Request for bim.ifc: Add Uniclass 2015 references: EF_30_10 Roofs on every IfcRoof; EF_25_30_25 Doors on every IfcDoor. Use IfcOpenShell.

First a look at what the model holds.

```python
import ifcopenshell

model = ifcopenshell.open("bim.ifc")
print(model.schema)
print("classifications:", [c.Name for c in model.by_type("IfcClassification")])
for ifc_class in ("IfcDoor", "IfcRoof", "IfcStair", "IfcWall", "IfcWindow"):
    print(ifc_class, len(model.by_type(ifc_class)))
```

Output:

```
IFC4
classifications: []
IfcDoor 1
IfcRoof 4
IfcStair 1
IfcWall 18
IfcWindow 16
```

```python
import ifcopenshell
import ifcopenshell.api.classification

model = ifcopenshell.open("bim.ifc")

system = ifcopenshell.api.classification.add_classification(model, classification="Uniclass 2015")

codes = {
    "IfcRoof": ("EF_30_10", "Roofs"),
    "IfcDoor": ("EF_25_30_25", "Doors"),
}
for ifc_class, (code, name) in codes.items():
    products = model.by_type(ifc_class)
    ifcopenshell.api.classification.add_reference(
        model, products=products, classification=system, identification=code, name=name
    )
    print(code, len(products))

model.write("bim-out.ifc")
```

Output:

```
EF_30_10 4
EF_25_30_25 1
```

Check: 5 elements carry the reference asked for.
